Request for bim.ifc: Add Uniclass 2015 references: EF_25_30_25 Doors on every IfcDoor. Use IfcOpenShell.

First a look at what the model holds.

```python
import ifcopenshell

model = ifcopenshell.open("bim.ifc")
print(model.schema)
print("classifications:", [c.Name for c in model.by_type("IfcClassification")])
for ifc_class in ("IfcDoor", "IfcRoof", "IfcStair", "IfcWall", "IfcWindow"):
    print(ifc_class, len(model.by_type(ifc_class)))
```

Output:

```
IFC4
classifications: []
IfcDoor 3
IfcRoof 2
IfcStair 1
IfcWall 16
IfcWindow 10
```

```python
import ifcopenshell
import ifcopenshell.api.classification

model = ifcopenshell.open("bim.ifc")

system = ifcopenshell.api.classification.add_classification(model, classification="Uniclass 2015")

codes = {
    "IfcDoor": ("EF_25_30_25", "Doors"),
}
for ifc_class, (code, name) in codes.items():
    products = model.by_type(ifc_class)
    ifcopenshell.api.classification.add_reference(
        model, products=products, classification=system, identification=code, name=name
    )
    print(code, len(products))

model.write("bim-out.ifc")
```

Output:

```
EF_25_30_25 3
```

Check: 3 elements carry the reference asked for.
